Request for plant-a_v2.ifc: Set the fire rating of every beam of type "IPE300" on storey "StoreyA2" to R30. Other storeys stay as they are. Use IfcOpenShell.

First a look at what the model holds.

```python
import ifcopenshell
import ifcopenshell.util.element

model = ifcopenshell.open("plant-a_v2.ifc")
print(model.schema)
storey = next(s for s in model.by_type("IfcBuildingStorey") if s.Name == "StoreyA2")
beams = [e for e in ifcopenshell.util.element.get_decomposition(storey) if e.is_a("IfcBeam")]
seen = {}
for e in beams:
    element_type = ifcopenshell.util.element.get_type(e)
    key = (element_type.Name if element_type != e and element_type else None, ifcopenshell.util.element.get_pset(e, "Pset_BeamCommon", "FireRating"))
    seen[key] = seen.get(key, 0) + 1
for (name, value), count in sorted(seen.items(), key=str):
    print(count, "x", name, "|", value)
```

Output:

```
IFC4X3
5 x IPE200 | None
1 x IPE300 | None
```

```python
import ifcopenshell
import ifcopenshell.api.pset
import ifcopenshell.util.element

model = ifcopenshell.open("plant-a_v2.ifc")

storey = next(s for s in model.by_type("IfcBuildingStorey") if s.Name == "StoreyA2")
beams = [e for e in ifcopenshell.util.element.get_decomposition(storey) if e.is_a("IfcBeam")]

count = 0
for e in beams:
    element_type = ifcopenshell.util.element.get_type(e)
    if element_type in (None, e) or element_type.Name != "IPE300":
        continue
    # add_pset returns the element's existing set when there is one.
    pset = ifcopenshell.api.pset.add_pset(model, product=e, name="Pset_BeamCommon")
    ifcopenshell.api.pset.edit_pset(model, pset=pset, properties={"FireRating": "R30"})
    count += 1

print(count, "beams updated")

model.write("plant-a_v2_updated.ifc")
```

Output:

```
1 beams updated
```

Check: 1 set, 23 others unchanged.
